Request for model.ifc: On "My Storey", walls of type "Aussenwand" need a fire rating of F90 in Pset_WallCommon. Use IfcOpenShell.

First a look at what the model holds.

```python
import ifcopenshell
import ifcopenshell.util.element

model = ifcopenshell.open("model.ifc")
print(model.schema)
storey = next(s for s in model.by_type("IfcBuildingStorey") if s.Name == "My Storey")
walls = [e for e in ifcopenshell.util.element.get_decomposition(storey) if e.is_a("IfcWall")]
seen = {}
for e in walls:
    element_type = ifcopenshell.util.element.get_type(e)
    key = (element_type.Name if element_type != e and element_type else None, ifcopenshell.util.element.get_pset(e, "Pset_WallCommon", "FireRating"))
    seen[key] = seen.get(key, 0) + 1
for (name, value), count in sorted(seen.items(), key=str):
    print(count, "x", name, "|", value)
```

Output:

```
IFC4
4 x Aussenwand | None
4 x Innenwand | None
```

```python
import ifcopenshell
import ifcopenshell.api.pset
import ifcopenshell.util.element

model = ifcopenshell.open("model.ifc")

storey = next(s for s in model.by_type("IfcBuildingStorey") if s.Name == "My Storey")
walls = [e for e in ifcopenshell.util.element.get_decomposition(storey) if e.is_a("IfcWall")]

count = 0
for e in walls:
    element_type = ifcopenshell.util.element.get_type(e)
    if element_type in (None, e) or element_type.Name != "Aussenwand":
        continue
    # add_pset returns the element's existing set when there is one.
    pset = ifcopenshell.api.pset.add_pset(model, product=e, name="Pset_WallCommon")
    ifcopenshell.api.pset.edit_pset(model, pset=pset, properties={"FireRating": "F90"})
    count += 1

print(count, "walls updated")

model.write("model_edited.ifc")
```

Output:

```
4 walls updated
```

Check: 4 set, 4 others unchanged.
